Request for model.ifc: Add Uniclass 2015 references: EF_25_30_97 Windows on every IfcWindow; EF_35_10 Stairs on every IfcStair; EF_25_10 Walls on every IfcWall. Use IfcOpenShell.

First a look at what the model holds.

```python
import ifcopenshell

model = ifcopenshell.open("model.ifc")
print(model.schema)
print("classifications:", [c.Name for c in model.by_type("IfcClassification")])
for ifc_class in ("IfcDoor", "IfcRoof", "IfcStair", "IfcWall", "IfcWindow"):
    print(ifc_class, len(model.by_type(ifc_class)))
```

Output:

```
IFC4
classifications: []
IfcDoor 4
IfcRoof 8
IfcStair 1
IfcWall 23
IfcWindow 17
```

```python
import ifcopenshell
import ifcopenshell.api.classification

model = ifcopenshell.open("model.ifc")

system = ifcopenshell.api.classification.add_classification(model, classification="Uniclass 2015")

codes = {
    "IfcWindow": ("EF_25_30_97", "Windows"),
    "IfcStair": ("EF_35_10", "Stairs"),
    "IfcWall": ("EF_25_10", "Walls"),
}
for ifc_class, (code, name) in codes.items():
    products = model.by_type(ifc_class)
    ifcopenshell.api.classification.add_reference(
        model, products=products, classification=system, identification=code, name=name
    )
    print(code, len(products))

model.write("model_edited.ifc")
```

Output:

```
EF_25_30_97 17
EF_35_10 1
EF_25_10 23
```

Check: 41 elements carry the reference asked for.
